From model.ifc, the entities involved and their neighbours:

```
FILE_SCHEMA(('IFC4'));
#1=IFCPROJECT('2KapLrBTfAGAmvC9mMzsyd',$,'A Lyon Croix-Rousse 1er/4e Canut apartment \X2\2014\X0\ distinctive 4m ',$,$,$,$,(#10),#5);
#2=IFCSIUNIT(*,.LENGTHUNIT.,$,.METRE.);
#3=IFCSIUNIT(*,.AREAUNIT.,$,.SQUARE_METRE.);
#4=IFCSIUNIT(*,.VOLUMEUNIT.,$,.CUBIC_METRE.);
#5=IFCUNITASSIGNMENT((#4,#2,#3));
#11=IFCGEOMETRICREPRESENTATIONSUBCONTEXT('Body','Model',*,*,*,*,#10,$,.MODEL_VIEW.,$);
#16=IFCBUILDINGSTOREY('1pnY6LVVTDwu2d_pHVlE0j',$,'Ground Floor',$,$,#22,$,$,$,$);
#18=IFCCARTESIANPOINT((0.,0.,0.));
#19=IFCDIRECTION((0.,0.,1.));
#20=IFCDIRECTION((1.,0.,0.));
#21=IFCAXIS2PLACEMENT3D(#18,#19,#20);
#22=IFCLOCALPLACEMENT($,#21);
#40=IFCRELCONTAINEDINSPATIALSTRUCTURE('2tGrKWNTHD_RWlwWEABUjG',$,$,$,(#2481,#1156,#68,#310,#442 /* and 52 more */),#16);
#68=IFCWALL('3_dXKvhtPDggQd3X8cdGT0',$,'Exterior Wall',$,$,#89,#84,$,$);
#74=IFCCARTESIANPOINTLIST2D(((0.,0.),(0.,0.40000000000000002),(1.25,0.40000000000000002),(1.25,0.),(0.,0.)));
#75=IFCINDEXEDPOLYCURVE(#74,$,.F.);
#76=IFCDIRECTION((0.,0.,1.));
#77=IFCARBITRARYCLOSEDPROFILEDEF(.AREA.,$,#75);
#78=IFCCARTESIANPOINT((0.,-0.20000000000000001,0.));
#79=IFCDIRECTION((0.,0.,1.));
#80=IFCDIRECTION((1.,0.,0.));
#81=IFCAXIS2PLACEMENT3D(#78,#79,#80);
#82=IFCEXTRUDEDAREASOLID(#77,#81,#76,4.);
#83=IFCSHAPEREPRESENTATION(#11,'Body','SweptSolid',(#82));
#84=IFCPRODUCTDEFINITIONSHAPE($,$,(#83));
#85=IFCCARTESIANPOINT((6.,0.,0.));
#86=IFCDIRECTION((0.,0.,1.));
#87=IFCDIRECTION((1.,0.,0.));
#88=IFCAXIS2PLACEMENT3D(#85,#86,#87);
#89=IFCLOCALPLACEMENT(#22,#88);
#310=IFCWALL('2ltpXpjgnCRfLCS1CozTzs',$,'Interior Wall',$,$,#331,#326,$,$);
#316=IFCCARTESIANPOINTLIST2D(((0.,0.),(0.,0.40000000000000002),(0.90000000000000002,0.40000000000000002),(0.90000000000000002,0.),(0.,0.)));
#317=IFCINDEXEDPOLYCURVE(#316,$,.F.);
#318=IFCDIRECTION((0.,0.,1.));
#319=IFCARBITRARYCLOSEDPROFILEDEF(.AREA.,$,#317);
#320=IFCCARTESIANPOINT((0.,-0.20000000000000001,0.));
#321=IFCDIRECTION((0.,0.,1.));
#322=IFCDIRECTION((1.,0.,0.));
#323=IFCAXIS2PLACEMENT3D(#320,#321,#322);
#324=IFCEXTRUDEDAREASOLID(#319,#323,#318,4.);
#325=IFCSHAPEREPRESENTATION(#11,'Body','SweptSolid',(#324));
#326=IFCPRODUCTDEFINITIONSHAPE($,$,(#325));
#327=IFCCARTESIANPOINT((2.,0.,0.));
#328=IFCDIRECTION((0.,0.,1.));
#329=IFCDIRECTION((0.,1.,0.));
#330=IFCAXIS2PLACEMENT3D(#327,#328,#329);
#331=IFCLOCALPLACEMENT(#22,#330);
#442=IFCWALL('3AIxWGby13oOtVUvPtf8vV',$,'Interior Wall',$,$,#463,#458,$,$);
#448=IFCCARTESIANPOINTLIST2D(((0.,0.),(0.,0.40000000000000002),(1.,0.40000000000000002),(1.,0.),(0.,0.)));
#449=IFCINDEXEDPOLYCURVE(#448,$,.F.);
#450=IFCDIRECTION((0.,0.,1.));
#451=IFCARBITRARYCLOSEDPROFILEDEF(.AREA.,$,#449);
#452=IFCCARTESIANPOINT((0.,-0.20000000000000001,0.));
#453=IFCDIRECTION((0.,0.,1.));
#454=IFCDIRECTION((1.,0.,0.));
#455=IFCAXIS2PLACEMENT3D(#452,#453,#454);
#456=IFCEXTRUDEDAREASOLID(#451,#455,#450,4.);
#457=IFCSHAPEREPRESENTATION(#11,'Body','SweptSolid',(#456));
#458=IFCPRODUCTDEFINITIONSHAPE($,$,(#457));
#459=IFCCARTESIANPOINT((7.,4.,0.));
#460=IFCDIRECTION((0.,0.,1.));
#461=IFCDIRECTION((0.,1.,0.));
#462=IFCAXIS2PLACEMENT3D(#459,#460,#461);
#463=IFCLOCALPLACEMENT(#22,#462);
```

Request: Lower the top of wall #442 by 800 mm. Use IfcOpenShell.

```python
import ifcopenshell
import ifcopenshell.geom
import ifcopenshell.util.representation
import ifcopenshell.util.shape
import ifcopenshell.util.unit

model = ifcopenshell.open("model.ifc")
unit_scale = ifcopenshell.util.unit.calculate_unit_scale(model)
settings = ifcopenshell.geom.settings()


def volume(element):
    """Net volume in cubic metres, openings subtracted."""
    shape = ifcopenshell.geom.create_shape(settings, element)
    return ifcopenshell.util.shape.get_volume(shape.geometry)


wall = model.by_guid("3AIxWGby13oOtVUvPtf8vV")
before = volume(wall)

body = ifcopenshell.util.representation.get_representation(wall, "Model", "Body")
solid = body.Items[0]
old_height = solid.Depth
solid.Depth -= 0.8 / unit_scale
after = volume(wall)

print(f"height {old_height:g} -> {solid.Depth:g}, volume {before:.3f} -> {after:.3f} m3")

model.write("model-out.ifc")
```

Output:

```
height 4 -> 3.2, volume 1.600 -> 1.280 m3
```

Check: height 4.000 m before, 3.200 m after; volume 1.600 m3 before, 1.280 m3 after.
